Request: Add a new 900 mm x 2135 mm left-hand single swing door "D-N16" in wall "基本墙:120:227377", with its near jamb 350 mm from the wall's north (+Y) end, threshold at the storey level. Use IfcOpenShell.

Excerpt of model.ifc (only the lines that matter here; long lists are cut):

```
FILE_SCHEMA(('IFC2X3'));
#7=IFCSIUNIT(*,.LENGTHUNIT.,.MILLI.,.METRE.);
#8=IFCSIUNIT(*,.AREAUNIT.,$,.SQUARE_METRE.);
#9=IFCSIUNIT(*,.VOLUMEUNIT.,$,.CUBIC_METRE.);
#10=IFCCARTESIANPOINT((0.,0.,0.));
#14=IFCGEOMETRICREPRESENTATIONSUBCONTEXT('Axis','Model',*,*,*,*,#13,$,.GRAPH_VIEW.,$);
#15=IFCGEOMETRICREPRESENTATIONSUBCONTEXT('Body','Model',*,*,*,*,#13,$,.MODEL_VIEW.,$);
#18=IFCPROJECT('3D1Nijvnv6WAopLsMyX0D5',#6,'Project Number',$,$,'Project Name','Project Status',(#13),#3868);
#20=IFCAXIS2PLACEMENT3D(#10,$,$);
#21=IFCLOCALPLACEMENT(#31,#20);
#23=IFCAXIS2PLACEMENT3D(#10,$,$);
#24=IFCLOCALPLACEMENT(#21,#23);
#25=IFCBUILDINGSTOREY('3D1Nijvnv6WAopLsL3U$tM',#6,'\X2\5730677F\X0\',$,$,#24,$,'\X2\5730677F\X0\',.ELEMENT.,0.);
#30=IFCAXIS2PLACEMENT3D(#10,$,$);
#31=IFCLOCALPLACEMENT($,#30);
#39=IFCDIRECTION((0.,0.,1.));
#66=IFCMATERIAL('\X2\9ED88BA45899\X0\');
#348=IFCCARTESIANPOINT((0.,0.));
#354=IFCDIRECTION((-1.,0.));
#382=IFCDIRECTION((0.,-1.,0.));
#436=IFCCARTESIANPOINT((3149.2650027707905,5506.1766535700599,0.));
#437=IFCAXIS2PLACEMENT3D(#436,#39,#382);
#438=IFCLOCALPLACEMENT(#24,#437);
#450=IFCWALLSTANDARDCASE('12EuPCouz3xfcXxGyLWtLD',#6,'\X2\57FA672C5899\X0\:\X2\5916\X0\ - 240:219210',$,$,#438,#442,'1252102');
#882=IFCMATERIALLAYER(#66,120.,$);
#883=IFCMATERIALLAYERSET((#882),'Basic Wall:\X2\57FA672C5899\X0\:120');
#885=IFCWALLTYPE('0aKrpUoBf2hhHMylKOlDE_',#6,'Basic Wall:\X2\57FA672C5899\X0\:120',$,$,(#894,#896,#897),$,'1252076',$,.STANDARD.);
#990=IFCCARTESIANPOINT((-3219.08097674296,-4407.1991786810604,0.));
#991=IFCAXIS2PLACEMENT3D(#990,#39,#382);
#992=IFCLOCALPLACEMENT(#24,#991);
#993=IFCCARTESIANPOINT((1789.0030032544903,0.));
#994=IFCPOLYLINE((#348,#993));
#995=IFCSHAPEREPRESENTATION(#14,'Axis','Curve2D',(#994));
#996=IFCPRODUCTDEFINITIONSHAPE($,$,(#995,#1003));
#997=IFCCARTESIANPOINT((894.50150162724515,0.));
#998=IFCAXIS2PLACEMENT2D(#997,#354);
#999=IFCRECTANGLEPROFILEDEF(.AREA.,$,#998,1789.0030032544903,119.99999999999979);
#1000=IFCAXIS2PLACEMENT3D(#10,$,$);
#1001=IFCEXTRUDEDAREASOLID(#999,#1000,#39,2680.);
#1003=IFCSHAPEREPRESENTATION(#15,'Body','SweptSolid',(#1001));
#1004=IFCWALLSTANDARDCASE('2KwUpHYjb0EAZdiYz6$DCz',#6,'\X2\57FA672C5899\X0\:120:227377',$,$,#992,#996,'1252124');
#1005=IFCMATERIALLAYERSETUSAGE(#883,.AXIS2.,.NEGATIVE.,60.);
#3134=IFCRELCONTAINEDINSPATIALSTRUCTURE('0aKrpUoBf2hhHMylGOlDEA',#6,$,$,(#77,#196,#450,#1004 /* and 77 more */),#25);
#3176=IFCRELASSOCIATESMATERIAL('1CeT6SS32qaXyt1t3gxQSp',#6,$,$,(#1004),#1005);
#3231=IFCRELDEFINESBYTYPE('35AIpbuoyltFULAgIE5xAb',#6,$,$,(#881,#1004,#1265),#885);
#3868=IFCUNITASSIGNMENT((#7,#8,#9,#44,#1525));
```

```python
import numpy as np
import ifcopenshell
import ifcopenshell.api.feature
import ifcopenshell.api.geometry
import ifcopenshell.api.root
import ifcopenshell.api.spatial
import ifcopenshell.api.type
import ifcopenshell.geom
import ifcopenshell.util.element
import ifcopenshell.util.placement
import ifcopenshell.util.representation
import ifcopenshell.util.shape
import ifcopenshell.util.unit

model = ifcopenshell.open("model.ifc")
unit_scale = ifcopenshell.util.unit.calculate_unit_scale(model)
settings = ifcopenshell.geom.settings()


def volume(element):
    """Net volume in cubic metres, openings subtracted."""
    shape = ifcopenshell.geom.create_shape(settings, element)
    return ifcopenshell.util.shape.get_volume(shape.geometry)


wall = model.by_guid("2KwUpHYjb0EAZdiYz6$DCz")
storey = ifcopenshell.util.element.get_container(wall, ifc_class="IfcBuildingStorey")
context = ifcopenshell.util.representation.get_context(model, "Model", "Body", "MODEL_VIEW")
before = volume(wall)

width, height, from_end, sill = 0.9, 2.135, 0.35, 0.0  # metres

# The wall runs along its own X axis, and the end named is its -X end.
wall_shape = ifcopenshell.geom.create_shape(settings, wall)
x, y, z = ifcopenshell.util.shape.get_vertices(wall_shape.geometry).T
start = x.min() + from_end
face, thickness = float(y.min()), float(y.max() - y.min())
wall_matrix = ifcopenshell.util.placement.get_local_placement(wall.ObjectPlacement)
level = ifcopenshell.util.placement.get_local_placement(storey.ObjectPlacement)[2, 3]


def in_wall(x, y):
    """Placement at x, y metres in the wall's axes, at sill height."""
    matrix = wall_matrix.copy()
    matrix[:, 3] = wall_matrix @ np.array([x / unit_scale, y / unit_scale, 0.0, 1.0])
    matrix[2, 3] = level + sill / unit_scale
    return matrix


# Opening: a box that overshoots both wall faces by 50 mm.
opening = ifcopenshell.api.root.create_entity(model, ifc_class="IfcOpeningElement")
box = ifcopenshell.api.geometry.add_wall_representation(
    model, context=context, length=width, height=height, thickness=thickness + 0.1
)
ifcopenshell.api.geometry.assign_representation(model, product=opening, representation=box)
ifcopenshell.api.geometry.edit_object_placement(model, product=opening, matrix=in_wall(start, face - 0.05), is_si=False)
ifcopenshell.api.feature.add_feature(model, feature=opening, element=wall)

door = ifcopenshell.api.root.create_entity(model, ifc_class="IfcDoor", name="D-N16")
door.OverallWidth, door.OverallHeight = width / unit_scale, height / unit_scale
body = ifcopenshell.api.geometry.add_door_representation(
    model,
    context=context,
    overall_width=door.OverallWidth,
    overall_height=door.OverallHeight,
    operation_type="SINGLE_SWING_LEFT",
    lining_properties={"LiningDepth": thickness / unit_scale, "ThresholdDepth": thickness / unit_scale},
)
ifcopenshell.api.geometry.assign_representation(model, product=door, representation=body)
ifcopenshell.api.spatial.assign_container(model, products=[door], relating_structure=storey)
fills = ifcopenshell.api.feature.add_filling(model, opening=opening, element=door)
fills.OwnerHistory = door.OwnerHistory  # required in IFC2X3

# IFC2X3 keeps the operation on the door style.
style = ifcopenshell.api.root.create_entity(model, ifc_class="IfcDoorStyle", name="D-N16")
style.OperationType, style.ConstructionType = "SINGLE_SWING_LEFT", "NOTDEFINED"
style.ParameterTakesPrecedence = style.Sizeable = False
ifcopenshell.api.type.assign_type(model, related_objects=[door], relating_type=style)

# The lining spans the wall, so the door starts at the wall face.
ifcopenshell.api.geometry.edit_object_placement(model, product=door, matrix=in_wall(start, face), is_si=False)

after = volume(wall)

print(f"wall volume {before:.3f} -> {after:.3f} m3")

model.write("model_edited.ifc")
```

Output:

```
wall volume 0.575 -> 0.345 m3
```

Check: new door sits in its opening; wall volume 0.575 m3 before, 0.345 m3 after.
